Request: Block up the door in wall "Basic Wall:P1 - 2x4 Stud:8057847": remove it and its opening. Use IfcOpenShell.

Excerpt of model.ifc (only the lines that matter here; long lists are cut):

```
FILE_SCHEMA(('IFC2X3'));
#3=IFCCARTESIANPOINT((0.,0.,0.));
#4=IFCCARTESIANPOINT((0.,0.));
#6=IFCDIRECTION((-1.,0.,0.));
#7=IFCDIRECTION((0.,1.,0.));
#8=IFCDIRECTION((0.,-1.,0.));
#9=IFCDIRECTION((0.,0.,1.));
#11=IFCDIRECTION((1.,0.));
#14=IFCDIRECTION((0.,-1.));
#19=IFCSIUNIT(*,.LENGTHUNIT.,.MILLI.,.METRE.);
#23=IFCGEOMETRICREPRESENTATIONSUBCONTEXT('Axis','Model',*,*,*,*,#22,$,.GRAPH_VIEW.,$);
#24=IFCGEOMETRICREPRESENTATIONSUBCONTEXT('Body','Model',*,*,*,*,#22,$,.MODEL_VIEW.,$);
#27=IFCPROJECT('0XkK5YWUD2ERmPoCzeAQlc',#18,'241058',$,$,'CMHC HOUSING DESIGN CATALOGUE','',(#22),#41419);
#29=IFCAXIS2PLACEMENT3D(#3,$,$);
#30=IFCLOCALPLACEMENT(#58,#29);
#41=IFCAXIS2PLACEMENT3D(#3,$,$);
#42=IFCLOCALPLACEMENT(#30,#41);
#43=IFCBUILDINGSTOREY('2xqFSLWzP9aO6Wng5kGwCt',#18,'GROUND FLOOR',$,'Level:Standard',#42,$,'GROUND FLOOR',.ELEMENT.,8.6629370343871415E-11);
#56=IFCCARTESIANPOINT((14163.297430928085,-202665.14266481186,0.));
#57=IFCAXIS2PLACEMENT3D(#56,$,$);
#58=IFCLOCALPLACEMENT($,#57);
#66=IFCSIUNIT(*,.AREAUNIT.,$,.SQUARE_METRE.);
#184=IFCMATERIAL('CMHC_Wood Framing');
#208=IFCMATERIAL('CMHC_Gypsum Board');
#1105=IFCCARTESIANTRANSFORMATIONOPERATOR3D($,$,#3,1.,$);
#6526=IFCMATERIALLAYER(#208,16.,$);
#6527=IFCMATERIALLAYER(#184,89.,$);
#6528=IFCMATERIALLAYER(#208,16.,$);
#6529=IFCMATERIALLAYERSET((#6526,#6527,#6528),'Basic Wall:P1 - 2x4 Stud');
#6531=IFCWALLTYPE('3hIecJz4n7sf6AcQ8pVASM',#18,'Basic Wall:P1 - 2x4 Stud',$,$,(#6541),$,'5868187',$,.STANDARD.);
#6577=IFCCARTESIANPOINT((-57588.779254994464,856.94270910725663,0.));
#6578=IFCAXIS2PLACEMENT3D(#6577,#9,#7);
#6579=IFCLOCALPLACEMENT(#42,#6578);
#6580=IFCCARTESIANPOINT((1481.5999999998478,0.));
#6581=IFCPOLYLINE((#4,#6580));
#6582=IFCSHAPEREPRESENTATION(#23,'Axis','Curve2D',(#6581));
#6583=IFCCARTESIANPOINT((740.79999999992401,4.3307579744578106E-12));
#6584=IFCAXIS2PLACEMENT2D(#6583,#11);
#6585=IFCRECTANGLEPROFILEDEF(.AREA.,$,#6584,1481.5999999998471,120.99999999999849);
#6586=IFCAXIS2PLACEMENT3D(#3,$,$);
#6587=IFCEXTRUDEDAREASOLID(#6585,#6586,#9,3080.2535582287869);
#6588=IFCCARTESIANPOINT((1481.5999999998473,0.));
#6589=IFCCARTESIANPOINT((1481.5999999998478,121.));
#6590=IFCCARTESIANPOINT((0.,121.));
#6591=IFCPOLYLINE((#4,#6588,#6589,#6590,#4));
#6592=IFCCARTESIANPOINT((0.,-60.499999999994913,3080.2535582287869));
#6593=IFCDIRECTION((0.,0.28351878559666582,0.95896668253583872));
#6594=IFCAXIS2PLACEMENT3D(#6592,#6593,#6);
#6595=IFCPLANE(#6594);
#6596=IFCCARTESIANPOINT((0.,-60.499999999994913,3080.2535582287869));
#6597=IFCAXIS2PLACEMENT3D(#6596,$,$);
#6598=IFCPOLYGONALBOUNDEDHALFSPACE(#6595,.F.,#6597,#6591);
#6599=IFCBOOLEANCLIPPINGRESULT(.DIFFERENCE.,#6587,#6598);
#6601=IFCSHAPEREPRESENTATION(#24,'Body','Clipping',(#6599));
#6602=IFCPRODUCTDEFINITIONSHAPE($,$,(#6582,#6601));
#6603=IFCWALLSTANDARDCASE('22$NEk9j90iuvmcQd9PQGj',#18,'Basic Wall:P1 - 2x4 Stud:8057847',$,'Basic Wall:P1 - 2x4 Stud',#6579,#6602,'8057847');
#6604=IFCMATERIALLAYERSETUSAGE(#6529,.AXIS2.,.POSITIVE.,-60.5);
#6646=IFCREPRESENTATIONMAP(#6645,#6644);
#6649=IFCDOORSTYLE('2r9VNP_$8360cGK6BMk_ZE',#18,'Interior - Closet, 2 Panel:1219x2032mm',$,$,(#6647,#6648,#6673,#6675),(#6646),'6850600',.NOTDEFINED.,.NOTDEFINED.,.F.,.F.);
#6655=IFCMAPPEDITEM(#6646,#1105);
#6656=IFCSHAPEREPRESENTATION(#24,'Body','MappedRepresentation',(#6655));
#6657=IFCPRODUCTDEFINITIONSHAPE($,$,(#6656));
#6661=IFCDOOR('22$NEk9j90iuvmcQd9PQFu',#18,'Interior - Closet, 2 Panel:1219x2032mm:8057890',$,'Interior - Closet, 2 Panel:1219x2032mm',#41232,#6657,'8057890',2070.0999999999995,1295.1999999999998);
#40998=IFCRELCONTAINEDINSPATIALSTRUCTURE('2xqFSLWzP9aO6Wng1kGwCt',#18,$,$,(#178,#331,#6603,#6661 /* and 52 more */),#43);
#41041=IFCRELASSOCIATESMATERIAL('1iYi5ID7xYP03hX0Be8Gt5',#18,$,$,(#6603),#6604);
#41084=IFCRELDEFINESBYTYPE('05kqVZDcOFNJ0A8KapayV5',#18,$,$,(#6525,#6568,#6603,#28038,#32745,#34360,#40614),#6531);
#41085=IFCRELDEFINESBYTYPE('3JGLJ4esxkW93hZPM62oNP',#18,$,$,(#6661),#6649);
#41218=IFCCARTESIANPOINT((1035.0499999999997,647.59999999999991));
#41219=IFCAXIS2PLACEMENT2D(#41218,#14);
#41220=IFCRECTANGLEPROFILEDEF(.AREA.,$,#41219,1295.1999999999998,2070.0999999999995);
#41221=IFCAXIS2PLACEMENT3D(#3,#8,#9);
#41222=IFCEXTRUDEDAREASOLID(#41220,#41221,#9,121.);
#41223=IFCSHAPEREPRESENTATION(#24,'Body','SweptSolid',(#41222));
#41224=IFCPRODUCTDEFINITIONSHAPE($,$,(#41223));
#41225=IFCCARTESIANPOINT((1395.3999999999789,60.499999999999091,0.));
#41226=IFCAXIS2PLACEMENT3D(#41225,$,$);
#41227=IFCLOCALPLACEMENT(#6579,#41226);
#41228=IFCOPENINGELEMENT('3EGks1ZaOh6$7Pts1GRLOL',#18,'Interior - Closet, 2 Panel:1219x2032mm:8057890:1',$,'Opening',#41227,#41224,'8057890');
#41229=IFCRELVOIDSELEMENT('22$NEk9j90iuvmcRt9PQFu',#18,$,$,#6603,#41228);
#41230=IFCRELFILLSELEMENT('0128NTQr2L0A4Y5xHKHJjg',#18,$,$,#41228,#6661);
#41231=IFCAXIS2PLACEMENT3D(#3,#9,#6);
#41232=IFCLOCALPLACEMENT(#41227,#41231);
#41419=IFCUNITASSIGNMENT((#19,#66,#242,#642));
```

```python
import ifcopenshell
import ifcopenshell.api.feature
import ifcopenshell.api.root
import ifcopenshell.geom
import ifcopenshell.util.shape

model = ifcopenshell.open("model.ifc")
settings = ifcopenshell.geom.settings()


def volume(element):
    """Net volume in cubic metres, openings subtracted."""
    shape = ifcopenshell.geom.create_shape(settings, element)
    return ifcopenshell.util.shape.get_volume(shape.geometry)


door = model.by_id(6661)
opening = door.FillsVoids[0].RelatingOpeningElement
wall = opening.VoidsElements[0].RelatingBuildingElement
before = volume(wall)

ifcopenshell.api.root.remove_product(model, product=door)
ifcopenshell.api.feature.remove_feature(model, feature=opening)

after = volume(wall)

print(f"wall volume {before:.3f} -> {after:.3f} m3")

model.write("model_edited.ifc")
```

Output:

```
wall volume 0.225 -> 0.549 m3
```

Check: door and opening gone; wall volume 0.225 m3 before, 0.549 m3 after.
